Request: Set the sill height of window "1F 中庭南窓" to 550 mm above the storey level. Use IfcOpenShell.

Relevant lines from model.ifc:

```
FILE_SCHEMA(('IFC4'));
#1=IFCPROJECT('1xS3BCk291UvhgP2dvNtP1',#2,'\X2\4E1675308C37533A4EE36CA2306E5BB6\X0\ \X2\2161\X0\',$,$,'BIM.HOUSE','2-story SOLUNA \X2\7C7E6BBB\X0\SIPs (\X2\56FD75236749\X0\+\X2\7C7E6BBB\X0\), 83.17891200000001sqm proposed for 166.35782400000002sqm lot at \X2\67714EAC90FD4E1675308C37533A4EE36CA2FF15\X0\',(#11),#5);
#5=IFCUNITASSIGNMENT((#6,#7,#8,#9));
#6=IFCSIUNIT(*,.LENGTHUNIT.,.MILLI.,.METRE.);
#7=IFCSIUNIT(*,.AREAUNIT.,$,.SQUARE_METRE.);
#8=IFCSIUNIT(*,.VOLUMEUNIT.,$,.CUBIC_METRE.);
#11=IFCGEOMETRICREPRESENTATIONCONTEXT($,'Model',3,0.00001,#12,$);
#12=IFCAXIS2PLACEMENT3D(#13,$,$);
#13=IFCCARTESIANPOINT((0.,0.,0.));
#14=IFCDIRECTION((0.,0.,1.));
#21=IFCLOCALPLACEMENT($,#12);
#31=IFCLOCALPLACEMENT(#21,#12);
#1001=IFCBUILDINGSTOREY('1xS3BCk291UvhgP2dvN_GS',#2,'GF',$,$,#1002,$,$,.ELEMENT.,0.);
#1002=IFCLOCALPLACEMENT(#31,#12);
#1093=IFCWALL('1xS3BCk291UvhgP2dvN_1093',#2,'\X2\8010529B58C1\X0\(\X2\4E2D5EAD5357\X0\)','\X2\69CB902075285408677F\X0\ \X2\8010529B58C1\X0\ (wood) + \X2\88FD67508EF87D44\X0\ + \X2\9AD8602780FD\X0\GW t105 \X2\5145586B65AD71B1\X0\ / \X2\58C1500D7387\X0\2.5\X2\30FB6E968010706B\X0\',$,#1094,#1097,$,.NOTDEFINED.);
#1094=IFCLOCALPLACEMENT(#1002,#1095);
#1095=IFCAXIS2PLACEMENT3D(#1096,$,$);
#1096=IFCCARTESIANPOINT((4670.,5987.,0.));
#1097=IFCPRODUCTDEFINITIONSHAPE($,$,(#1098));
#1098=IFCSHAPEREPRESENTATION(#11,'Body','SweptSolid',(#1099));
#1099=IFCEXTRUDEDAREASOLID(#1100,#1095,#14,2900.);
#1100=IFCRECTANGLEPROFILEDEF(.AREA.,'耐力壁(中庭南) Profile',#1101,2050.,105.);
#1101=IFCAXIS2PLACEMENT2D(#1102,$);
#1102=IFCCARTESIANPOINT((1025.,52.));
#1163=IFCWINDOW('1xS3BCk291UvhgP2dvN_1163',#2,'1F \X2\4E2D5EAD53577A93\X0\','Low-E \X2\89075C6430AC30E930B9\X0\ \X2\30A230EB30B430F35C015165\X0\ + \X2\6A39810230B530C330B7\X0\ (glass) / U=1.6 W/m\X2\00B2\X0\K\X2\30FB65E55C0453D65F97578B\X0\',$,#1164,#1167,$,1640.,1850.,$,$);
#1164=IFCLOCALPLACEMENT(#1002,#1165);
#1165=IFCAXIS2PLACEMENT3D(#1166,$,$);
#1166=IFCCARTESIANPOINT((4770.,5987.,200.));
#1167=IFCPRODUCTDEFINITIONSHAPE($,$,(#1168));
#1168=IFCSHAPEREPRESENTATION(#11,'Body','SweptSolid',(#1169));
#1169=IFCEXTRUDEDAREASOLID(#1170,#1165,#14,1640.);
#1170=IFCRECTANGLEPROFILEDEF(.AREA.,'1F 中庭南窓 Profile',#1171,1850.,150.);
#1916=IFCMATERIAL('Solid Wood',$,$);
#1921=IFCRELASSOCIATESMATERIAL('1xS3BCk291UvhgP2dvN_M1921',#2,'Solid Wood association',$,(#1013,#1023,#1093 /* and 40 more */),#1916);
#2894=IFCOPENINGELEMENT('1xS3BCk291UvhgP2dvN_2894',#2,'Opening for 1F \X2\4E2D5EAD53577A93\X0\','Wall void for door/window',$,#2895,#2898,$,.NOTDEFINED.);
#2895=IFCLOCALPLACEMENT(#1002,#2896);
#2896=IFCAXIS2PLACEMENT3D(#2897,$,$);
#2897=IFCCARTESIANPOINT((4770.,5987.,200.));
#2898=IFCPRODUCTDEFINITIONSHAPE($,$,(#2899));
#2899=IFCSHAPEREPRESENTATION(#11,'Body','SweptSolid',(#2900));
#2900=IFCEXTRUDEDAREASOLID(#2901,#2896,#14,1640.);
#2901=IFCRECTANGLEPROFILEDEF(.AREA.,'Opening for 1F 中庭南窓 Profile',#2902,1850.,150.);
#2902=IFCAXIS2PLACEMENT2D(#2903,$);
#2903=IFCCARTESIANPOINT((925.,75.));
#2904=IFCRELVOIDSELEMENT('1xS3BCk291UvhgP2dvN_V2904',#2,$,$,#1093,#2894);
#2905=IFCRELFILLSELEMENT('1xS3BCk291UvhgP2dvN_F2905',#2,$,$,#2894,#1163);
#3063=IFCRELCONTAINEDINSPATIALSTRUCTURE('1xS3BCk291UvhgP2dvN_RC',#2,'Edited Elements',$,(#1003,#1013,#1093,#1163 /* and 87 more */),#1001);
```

```python
import numpy as np
import ifcopenshell
import ifcopenshell.api.geometry
import ifcopenshell.geom
import ifcopenshell.util.element
import ifcopenshell.util.placement
import ifcopenshell.util.shape
import ifcopenshell.util.unit

model = ifcopenshell.open("model.ifc")
unit_scale = ifcopenshell.util.unit.calculate_unit_scale(model)

window = model.by_id(1163)
opening = window.FillsVoids[0].RelatingOpeningElement
storey = ifcopenshell.util.element.get_container(window, ifc_class="IfcBuildingStorey")
level = ifcopenshell.util.placement.get_local_placement(storey.ObjectPlacement)[2, 3]

# The opening's origin need not be at the sill, so measure its lowest point.
shape = ifcopenshell.geom.create_shape(ifcopenshell.geom.settings(), opening)
bottom = ifcopenshell.util.shape.get_shape_bottom_elevation(shape, shape.geometry) / unit_scale
dz = level + 0.55 / unit_scale - bottom

shift = np.array([0.0, 0.0, dz])
# The window is not placed relative to its opening, so move both.
for product in (opening, window):
    matrix = ifcopenshell.util.placement.get_local_placement(product.ObjectPlacement)
    matrix[:3, 3] += shift
    ifcopenshell.api.geometry.edit_object_placement(model, product=product, matrix=matrix, is_si=False)

print(f"moved by {dz * unit_scale:+.3f} m")

model.write("model-out.ifc")
```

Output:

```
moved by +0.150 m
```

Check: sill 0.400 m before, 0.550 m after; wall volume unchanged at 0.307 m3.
